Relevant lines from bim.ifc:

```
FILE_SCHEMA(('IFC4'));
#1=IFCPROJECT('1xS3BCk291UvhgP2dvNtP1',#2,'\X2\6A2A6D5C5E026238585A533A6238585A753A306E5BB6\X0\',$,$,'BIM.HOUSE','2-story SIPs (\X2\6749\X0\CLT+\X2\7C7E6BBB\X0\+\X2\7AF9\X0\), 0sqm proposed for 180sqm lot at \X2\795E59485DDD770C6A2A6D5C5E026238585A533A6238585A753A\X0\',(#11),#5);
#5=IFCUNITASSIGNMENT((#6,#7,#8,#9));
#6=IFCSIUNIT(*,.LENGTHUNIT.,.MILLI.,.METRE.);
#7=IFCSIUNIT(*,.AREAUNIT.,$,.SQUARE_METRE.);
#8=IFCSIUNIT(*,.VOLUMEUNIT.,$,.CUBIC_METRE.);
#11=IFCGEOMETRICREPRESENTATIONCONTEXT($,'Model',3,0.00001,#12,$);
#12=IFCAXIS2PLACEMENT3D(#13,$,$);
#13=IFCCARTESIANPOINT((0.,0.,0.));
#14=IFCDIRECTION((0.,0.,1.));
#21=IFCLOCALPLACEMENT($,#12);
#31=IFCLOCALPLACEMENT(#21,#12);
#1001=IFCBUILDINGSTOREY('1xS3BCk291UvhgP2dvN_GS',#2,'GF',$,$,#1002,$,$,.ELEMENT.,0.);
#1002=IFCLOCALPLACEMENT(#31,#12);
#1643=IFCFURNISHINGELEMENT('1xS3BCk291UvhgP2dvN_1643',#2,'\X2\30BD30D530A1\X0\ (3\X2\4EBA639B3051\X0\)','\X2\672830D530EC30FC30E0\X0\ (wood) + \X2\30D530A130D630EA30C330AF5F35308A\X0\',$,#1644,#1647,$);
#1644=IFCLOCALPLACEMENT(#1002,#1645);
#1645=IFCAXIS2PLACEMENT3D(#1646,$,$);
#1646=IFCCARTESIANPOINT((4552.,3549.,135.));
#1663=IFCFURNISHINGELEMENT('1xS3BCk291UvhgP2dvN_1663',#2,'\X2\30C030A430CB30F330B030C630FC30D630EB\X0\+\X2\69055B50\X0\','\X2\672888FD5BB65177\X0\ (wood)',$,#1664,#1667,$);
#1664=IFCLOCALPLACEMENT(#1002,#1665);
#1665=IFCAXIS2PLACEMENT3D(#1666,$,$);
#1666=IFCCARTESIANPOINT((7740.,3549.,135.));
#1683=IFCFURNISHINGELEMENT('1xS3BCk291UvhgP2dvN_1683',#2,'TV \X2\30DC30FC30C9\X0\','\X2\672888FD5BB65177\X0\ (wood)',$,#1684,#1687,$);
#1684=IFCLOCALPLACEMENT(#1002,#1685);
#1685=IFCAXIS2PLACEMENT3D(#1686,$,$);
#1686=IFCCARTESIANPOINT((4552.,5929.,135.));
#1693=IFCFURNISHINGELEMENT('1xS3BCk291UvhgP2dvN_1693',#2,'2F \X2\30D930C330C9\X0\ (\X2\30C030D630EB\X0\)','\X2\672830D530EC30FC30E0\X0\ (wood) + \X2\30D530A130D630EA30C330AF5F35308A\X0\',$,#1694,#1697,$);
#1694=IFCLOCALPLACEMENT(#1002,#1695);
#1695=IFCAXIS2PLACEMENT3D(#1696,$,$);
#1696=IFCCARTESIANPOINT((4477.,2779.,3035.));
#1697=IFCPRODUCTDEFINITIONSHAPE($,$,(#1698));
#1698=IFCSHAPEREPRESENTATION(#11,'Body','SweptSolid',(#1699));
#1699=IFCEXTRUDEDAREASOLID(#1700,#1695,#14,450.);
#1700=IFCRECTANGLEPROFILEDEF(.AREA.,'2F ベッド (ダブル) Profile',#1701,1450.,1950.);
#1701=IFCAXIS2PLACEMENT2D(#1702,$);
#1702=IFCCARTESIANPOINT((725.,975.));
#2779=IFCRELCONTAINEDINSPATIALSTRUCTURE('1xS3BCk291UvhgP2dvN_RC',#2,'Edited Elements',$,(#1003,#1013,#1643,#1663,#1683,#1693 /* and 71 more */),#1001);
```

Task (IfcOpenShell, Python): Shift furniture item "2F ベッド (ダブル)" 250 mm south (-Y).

```python
import ifcopenshell
import ifcopenshell.api.geometry
import ifcopenshell.util.placement
import ifcopenshell.util.unit

model = ifcopenshell.open("bim.ifc")
unit_scale = ifcopenshell.util.unit.calculate_unit_scale(model)

item = model.by_id(1693)
matrix = ifcopenshell.util.placement.get_local_placement(item.ObjectPlacement)
matrix[1, 3] -= 0.25 / unit_scale
ifcopenshell.api.geometry.edit_object_placement(model, product=item, matrix=matrix, is_si=False)

print(ifcopenshell.util.placement.get_local_placement(item.ObjectPlacement).round(3) + 0.0)

model.write("bim_edited.ifc")
```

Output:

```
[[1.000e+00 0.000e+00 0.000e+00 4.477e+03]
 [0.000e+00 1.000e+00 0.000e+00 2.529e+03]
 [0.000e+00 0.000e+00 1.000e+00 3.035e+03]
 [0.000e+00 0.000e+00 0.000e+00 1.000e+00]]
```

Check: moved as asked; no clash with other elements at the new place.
